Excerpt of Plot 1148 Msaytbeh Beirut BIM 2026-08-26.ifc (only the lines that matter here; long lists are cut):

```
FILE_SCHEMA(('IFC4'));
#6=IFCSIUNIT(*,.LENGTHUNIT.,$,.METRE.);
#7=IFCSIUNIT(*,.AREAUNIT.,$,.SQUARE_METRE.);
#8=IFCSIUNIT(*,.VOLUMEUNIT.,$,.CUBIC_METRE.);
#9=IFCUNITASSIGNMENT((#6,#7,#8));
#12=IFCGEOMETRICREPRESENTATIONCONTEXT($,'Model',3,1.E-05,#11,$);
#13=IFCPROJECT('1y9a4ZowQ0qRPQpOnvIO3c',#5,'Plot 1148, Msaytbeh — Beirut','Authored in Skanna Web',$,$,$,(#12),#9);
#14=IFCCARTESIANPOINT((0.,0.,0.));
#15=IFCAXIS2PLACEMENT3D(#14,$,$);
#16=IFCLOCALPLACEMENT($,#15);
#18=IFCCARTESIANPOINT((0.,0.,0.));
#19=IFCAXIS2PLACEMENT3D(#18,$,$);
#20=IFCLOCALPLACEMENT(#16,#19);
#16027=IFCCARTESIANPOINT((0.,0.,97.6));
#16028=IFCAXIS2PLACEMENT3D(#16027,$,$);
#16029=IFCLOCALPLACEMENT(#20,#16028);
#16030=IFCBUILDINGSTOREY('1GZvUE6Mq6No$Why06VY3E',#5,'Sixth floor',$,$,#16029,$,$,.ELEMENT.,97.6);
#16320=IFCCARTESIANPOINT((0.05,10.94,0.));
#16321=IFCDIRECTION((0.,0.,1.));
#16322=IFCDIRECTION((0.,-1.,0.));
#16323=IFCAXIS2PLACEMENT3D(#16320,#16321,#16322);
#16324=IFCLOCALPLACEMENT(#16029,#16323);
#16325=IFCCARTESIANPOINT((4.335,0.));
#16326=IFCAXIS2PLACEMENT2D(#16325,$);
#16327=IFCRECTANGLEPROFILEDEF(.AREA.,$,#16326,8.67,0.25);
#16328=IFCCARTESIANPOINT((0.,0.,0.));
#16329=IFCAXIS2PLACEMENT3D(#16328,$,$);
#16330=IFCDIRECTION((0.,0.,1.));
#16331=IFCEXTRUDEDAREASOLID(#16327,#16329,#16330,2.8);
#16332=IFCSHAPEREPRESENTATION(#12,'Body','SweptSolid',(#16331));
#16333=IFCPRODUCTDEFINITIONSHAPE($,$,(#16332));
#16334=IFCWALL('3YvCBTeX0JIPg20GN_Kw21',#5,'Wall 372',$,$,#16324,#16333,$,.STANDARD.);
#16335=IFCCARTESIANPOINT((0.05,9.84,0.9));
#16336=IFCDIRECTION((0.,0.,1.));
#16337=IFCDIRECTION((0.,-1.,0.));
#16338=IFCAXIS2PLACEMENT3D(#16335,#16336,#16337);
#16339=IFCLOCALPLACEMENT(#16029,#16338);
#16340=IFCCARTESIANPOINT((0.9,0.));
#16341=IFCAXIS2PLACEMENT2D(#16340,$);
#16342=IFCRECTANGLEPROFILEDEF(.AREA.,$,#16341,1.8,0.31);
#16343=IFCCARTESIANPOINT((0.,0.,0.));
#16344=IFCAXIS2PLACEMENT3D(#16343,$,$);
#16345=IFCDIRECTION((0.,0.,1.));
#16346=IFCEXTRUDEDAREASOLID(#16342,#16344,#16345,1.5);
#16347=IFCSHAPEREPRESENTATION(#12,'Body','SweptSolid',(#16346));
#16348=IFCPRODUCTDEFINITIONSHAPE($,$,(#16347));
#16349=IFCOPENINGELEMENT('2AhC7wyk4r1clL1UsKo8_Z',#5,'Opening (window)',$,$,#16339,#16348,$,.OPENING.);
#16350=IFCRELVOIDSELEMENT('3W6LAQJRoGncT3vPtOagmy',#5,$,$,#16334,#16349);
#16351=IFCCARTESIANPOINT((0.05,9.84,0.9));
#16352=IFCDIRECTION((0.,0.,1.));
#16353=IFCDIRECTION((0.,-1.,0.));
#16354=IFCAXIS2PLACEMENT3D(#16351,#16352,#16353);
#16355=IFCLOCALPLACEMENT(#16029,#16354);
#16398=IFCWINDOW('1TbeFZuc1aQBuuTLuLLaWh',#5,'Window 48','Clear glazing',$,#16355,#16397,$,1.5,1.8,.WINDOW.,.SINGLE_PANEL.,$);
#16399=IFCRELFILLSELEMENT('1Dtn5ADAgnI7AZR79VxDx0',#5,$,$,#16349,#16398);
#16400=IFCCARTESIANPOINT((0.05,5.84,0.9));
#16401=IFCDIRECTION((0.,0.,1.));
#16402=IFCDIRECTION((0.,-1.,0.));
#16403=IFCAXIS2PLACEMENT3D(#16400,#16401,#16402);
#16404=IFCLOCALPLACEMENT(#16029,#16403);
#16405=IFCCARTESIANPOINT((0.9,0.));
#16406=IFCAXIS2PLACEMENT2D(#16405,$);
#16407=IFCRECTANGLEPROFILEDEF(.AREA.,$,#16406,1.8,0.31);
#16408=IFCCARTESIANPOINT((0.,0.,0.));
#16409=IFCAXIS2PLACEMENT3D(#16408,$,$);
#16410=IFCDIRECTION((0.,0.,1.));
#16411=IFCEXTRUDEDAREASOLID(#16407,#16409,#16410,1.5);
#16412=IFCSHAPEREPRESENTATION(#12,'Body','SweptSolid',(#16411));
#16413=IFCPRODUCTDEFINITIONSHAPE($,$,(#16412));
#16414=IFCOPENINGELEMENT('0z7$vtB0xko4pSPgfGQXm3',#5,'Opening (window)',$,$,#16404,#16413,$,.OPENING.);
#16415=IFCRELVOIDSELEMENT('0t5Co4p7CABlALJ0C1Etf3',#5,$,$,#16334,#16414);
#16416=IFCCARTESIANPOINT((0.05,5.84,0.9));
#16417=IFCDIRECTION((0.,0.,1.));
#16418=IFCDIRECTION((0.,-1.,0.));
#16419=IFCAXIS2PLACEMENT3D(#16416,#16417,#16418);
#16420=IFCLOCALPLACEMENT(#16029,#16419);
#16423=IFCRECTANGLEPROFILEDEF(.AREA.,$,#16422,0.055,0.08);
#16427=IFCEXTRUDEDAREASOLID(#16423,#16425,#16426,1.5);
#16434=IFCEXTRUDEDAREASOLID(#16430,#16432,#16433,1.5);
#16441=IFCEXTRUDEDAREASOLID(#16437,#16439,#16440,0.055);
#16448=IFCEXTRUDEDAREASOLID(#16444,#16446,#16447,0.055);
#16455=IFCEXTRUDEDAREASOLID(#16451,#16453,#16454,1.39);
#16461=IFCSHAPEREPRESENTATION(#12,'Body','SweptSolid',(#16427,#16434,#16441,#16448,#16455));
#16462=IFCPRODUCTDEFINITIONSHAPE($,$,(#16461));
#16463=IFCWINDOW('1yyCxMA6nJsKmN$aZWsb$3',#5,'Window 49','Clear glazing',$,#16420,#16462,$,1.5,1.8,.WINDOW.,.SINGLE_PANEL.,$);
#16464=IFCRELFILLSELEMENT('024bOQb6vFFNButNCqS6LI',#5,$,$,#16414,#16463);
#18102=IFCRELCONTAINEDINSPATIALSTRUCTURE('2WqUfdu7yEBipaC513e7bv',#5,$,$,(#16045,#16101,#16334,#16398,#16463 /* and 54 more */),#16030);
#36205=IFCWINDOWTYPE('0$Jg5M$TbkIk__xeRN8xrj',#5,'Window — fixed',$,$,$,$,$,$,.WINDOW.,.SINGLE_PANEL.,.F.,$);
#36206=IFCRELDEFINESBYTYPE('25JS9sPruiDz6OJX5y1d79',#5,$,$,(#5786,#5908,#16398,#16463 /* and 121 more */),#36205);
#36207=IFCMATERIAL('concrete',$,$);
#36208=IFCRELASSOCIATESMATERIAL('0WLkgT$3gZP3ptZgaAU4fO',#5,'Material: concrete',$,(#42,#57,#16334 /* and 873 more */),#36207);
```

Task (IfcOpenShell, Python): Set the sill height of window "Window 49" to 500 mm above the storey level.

```python
import numpy as np
import ifcopenshell
import ifcopenshell.api.geometry
import ifcopenshell.geom
import ifcopenshell.util.element
import ifcopenshell.util.placement
import ifcopenshell.util.shape
import ifcopenshell.util.unit

model = ifcopenshell.open("Plot 1148 Msaytbeh Beirut BIM 2026-08-26.ifc")
unit_scale = ifcopenshell.util.unit.calculate_unit_scale(model)

window = model.by_guid("1yyCxMA6nJsKmN$aZWsb$3")
opening = window.FillsVoids[0].RelatingOpeningElement
storey = ifcopenshell.util.element.get_container(window, ifc_class="IfcBuildingStorey")
level = ifcopenshell.util.placement.get_local_placement(storey.ObjectPlacement)[2, 3]

# The opening's origin need not be at the sill, so measure its lowest point.
shape = ifcopenshell.geom.create_shape(ifcopenshell.geom.settings(), opening)
bottom = ifcopenshell.util.shape.get_shape_bottom_elevation(shape, shape.geometry) / unit_scale
dz = level + 0.5 / unit_scale - bottom

shift = np.array([0.0, 0.0, dz])
# The window is not placed relative to its opening, so move both.
for product in (opening, window):
    matrix = ifcopenshell.util.placement.get_local_placement(product.ObjectPlacement)
    matrix[:3, 3] += shift
    ifcopenshell.api.geometry.edit_object_placement(model, product=product, matrix=matrix, is_si=False)

print(f"moved by {dz * unit_scale:+.3f} m")

model.write("Plot 1148 Msaytbeh Beirut BIM 2026-08-26_v2.ifc")
```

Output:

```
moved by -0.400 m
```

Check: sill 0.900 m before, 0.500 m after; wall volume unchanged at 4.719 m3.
